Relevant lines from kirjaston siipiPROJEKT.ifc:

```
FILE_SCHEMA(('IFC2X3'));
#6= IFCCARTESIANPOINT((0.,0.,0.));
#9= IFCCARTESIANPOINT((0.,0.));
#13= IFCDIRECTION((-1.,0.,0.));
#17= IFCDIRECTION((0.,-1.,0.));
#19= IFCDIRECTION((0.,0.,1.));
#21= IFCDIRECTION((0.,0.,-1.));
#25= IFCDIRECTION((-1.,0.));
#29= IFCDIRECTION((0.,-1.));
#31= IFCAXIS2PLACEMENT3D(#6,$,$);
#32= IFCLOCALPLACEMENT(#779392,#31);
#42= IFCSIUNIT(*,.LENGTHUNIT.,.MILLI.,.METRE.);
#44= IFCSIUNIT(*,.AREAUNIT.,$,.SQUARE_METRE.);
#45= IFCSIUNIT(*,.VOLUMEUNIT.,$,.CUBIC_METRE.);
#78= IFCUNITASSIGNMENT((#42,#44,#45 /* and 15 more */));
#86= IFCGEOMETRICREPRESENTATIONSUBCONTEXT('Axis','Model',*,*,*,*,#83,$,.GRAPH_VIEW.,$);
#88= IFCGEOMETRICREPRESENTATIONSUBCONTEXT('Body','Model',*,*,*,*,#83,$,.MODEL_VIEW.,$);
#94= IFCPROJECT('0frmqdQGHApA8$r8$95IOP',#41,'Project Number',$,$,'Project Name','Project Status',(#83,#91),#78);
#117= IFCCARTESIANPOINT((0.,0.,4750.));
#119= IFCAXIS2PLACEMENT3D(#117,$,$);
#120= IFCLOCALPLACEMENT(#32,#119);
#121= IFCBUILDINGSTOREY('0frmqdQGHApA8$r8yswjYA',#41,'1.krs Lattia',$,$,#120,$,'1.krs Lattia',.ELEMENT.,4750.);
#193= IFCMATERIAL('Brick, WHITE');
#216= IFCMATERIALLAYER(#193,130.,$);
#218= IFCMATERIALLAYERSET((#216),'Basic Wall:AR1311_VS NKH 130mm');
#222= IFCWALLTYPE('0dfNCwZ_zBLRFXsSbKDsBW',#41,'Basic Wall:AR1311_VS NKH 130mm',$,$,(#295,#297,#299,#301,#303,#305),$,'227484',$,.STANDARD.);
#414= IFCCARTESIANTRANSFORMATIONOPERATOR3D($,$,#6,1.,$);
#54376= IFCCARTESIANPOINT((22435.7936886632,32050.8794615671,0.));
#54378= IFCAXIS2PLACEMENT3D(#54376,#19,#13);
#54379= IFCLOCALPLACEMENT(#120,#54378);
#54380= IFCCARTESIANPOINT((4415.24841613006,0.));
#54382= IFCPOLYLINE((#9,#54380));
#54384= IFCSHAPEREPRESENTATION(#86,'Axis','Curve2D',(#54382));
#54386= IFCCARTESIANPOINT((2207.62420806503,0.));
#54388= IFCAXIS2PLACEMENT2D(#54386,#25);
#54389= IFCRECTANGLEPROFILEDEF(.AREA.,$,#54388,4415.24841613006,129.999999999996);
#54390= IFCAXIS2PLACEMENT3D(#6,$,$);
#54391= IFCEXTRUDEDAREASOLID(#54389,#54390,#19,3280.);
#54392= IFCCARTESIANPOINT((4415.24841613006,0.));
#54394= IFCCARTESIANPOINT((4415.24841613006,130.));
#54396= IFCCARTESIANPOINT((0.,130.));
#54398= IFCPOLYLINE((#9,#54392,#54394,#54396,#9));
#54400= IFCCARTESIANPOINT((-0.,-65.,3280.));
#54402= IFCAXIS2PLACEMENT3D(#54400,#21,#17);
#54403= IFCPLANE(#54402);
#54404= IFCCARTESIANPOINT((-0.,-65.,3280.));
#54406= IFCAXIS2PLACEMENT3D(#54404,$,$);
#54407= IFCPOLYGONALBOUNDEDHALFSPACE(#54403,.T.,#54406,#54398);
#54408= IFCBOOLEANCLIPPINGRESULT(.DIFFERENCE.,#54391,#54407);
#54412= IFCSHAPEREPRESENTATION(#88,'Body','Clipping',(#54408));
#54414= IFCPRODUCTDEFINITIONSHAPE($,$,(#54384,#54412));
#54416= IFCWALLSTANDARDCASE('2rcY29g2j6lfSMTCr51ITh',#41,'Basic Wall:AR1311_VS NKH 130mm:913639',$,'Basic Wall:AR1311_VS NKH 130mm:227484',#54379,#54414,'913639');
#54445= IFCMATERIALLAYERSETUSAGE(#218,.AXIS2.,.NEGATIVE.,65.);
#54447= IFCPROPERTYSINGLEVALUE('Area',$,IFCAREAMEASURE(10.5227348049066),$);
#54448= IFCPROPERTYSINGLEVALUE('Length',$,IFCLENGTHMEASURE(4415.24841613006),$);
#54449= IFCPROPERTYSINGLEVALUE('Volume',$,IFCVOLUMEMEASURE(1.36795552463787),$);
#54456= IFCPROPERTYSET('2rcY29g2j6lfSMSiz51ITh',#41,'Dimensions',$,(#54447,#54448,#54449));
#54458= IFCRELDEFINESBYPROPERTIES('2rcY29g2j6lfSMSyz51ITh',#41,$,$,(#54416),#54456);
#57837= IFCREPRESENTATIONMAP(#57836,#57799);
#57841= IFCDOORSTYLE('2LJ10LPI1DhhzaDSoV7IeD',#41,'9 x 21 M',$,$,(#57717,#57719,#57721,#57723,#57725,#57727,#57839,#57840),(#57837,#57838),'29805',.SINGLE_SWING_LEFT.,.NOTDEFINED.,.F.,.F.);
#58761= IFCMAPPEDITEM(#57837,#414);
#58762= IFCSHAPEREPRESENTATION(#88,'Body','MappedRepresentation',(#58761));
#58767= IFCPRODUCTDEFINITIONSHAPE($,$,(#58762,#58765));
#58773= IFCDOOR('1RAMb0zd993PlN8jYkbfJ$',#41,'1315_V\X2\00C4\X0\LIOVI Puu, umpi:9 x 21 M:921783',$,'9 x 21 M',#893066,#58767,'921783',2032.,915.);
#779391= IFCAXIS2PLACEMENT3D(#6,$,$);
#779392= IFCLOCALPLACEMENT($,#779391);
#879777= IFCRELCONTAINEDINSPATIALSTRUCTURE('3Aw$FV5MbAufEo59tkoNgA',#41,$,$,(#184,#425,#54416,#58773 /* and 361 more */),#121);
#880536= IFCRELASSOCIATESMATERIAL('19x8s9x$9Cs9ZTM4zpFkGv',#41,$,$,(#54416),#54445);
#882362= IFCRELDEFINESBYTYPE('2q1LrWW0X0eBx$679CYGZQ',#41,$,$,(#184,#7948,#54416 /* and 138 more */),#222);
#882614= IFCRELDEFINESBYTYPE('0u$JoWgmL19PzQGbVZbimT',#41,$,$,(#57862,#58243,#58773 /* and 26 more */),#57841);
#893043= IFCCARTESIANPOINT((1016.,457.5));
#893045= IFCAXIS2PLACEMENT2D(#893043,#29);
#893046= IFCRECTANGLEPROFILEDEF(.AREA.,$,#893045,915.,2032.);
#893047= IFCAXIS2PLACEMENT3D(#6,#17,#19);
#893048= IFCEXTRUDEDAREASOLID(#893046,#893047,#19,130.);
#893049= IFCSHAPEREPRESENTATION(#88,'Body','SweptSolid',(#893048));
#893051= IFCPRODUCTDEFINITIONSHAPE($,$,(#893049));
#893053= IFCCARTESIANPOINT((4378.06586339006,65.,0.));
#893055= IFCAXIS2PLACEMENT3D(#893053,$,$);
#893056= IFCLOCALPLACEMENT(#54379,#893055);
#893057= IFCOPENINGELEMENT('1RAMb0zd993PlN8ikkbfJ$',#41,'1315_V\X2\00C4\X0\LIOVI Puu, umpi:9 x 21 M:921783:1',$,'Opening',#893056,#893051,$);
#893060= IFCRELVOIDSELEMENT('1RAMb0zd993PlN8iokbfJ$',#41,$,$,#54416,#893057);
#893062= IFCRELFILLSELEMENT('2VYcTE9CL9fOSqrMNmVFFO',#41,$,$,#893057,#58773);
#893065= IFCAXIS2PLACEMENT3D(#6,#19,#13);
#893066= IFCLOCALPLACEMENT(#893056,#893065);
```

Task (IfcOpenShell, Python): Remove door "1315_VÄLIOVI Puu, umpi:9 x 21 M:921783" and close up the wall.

```python
import ifcopenshell
import ifcopenshell.api.feature
import ifcopenshell.api.pset
import ifcopenshell.api.root
import ifcopenshell.geom
import ifcopenshell.util.element
import ifcopenshell.util.shape
import ifcopenshell.util.unit

model = ifcopenshell.open("kirjaston siipiPROJEKT.ifc")
area_scale = ifcopenshell.util.unit.calculate_unit_scale(model, "AREAUNIT")
volume_scale = ifcopenshell.util.unit.calculate_unit_scale(model, "VOLUMEUNIT")
settings = ifcopenshell.geom.settings()


def volume(element):
    """Net volume in cubic metres, openings subtracted."""
    shape = ifcopenshell.geom.create_shape(settings, element)
    return ifcopenshell.util.shape.get_volume(shape.geometry)


door = model.by_guid("1RAMb0zd993PlN8jYkbfJ$")
opening = door.FillsVoids[0].RelatingOpeningElement
wall = opening.VoidsElements[0].RelatingBuildingElement
before = volume(wall)

ifcopenshell.api.root.remove_product(model, product=door)
ifcopenshell.api.feature.remove_feature(model, feature=opening)

after = volume(wall)
thickness = 0.13  # wall thickness in metres

# Update the wall's stored quantities.
pset = model.by_id(ifcopenshell.util.element.get_pset(wall, "Dimensions", should_inherit=False)["id"])
ifcopenshell.api.pset.edit_pset(model, pset=pset, properties={
    "Area": model.create_entity("IfcAreaMeasure", after / thickness / area_scale),
    "Volume": model.create_entity("IfcVolumeMeasure", after / volume_scale),
})

print(f"wall volume {before:.3f} -> {after:.3f} m3")

model.write("kirjaston siipiPROJEKT_updated.ifc")
```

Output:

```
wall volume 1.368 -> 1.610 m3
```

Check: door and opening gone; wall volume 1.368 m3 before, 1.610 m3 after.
